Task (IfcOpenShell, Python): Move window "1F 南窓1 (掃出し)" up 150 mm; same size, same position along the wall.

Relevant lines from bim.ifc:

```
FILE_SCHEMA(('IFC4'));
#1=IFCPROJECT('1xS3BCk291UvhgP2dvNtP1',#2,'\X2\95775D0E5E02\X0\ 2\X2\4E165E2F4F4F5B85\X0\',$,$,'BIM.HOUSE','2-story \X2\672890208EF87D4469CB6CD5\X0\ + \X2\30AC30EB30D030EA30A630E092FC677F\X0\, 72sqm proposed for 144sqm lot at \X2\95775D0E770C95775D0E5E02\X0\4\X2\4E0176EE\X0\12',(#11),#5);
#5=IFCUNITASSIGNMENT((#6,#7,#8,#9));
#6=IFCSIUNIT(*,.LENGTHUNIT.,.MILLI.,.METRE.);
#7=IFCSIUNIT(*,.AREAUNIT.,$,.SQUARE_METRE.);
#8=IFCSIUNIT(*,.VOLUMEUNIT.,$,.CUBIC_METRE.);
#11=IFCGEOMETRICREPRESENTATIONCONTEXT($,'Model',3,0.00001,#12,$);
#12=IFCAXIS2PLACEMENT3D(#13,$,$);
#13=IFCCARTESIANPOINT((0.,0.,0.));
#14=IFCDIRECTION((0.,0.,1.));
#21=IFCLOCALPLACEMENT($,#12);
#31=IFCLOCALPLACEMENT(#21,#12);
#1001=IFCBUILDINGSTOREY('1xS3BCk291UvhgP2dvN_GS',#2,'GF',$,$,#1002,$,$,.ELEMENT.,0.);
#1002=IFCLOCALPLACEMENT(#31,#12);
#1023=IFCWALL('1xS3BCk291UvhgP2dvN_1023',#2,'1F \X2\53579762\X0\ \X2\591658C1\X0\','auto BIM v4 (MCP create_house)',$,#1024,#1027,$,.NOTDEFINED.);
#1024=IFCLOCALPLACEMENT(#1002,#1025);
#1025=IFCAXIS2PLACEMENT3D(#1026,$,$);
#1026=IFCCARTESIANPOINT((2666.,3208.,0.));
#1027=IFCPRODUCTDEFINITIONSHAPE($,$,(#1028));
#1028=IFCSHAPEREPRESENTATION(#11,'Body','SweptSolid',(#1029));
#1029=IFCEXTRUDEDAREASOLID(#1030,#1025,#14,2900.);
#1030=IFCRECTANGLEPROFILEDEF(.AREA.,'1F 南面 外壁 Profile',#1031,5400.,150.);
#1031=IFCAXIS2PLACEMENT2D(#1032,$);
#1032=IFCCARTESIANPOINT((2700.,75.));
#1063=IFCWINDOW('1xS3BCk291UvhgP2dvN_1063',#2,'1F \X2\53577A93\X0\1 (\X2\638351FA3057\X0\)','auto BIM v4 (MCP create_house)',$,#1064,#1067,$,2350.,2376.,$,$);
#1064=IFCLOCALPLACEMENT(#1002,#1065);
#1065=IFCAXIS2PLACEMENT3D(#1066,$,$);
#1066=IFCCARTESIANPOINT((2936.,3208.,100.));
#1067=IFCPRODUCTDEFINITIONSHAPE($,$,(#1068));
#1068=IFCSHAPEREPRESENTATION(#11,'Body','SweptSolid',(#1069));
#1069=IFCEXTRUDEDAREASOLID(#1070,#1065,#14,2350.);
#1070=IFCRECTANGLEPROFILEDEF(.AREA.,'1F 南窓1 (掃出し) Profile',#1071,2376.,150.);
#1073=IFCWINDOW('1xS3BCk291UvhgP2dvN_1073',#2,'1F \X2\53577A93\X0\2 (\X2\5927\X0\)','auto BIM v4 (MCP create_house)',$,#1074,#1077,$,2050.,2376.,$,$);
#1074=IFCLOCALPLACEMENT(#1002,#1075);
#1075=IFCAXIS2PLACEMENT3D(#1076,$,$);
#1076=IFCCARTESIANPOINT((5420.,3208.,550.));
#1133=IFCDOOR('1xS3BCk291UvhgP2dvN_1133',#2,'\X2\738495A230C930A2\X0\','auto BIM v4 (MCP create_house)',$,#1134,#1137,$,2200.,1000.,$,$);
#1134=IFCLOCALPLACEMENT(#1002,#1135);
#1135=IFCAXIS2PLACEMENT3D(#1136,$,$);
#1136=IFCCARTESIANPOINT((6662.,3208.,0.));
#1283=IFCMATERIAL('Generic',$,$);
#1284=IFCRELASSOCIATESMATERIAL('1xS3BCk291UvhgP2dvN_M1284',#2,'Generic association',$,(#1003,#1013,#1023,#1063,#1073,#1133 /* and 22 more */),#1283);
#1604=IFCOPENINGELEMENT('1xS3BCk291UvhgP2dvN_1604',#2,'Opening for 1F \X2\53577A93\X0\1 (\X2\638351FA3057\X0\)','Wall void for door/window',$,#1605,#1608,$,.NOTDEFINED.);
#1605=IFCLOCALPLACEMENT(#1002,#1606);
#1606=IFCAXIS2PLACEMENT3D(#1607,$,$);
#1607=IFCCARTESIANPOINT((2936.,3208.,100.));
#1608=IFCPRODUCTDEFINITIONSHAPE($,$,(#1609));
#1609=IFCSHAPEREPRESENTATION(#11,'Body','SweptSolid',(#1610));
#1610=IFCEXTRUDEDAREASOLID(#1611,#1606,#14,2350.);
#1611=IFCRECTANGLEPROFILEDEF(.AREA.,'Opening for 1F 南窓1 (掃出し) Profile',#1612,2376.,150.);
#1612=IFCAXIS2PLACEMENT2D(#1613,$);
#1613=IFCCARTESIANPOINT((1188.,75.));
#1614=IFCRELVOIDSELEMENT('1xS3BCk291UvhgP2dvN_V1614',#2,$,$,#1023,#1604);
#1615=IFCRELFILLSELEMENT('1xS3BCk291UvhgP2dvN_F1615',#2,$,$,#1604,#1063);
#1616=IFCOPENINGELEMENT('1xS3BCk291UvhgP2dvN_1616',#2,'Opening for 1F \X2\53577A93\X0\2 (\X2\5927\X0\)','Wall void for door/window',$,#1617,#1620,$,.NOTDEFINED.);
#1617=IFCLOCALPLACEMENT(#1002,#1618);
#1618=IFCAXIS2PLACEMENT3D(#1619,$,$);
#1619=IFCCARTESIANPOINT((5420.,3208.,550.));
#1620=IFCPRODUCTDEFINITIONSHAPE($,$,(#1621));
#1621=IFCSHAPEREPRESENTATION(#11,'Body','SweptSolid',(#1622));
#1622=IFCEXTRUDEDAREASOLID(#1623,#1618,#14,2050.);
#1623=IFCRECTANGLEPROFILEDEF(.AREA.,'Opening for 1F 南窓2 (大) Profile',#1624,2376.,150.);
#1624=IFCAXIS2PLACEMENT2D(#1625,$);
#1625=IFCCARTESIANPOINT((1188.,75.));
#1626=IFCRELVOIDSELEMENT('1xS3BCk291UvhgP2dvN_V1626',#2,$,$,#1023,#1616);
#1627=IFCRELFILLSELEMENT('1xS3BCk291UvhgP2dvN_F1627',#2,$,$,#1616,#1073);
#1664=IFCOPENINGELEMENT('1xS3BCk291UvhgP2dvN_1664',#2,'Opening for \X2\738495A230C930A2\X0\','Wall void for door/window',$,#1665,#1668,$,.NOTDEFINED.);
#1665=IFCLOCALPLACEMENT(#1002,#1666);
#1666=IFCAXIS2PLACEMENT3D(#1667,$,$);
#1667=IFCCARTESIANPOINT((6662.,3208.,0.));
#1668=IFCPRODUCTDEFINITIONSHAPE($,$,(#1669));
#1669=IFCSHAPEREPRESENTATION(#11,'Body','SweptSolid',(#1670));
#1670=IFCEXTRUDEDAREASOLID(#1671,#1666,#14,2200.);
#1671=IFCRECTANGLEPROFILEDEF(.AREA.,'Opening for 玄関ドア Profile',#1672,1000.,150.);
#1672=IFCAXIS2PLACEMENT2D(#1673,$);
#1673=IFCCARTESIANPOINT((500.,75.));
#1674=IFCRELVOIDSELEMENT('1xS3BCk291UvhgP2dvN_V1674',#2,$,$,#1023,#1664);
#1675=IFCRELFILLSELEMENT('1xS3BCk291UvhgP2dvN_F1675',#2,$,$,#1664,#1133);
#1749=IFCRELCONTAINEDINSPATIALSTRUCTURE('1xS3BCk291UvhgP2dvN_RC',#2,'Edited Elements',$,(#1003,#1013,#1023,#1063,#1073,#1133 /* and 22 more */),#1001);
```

```python
import numpy as np
import ifcopenshell
import ifcopenshell.api.geometry
import ifcopenshell.util.placement
import ifcopenshell.util.unit

model = ifcopenshell.open("bim.ifc")
unit_scale = ifcopenshell.util.unit.calculate_unit_scale(model)

window = model.by_guid("1xS3BCk291UvhgP2dvN_1063")
opening = window.FillsVoids[0].RelatingOpeningElement
dz = 150.0

shift = np.array([0.0, 0.0, dz])
# The window is not placed relative to its opening, so move both.
for product in (opening, window):
    matrix = ifcopenshell.util.placement.get_local_placement(product.ObjectPlacement)
    matrix[:3, 3] += shift
    ifcopenshell.api.geometry.edit_object_placement(model, product=product, matrix=matrix, is_si=False)

print(f"moved by {dz * unit_scale:+.3f} m")

model.write("bim_rev.ifc")
```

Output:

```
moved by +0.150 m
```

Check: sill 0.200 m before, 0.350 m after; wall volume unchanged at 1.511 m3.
